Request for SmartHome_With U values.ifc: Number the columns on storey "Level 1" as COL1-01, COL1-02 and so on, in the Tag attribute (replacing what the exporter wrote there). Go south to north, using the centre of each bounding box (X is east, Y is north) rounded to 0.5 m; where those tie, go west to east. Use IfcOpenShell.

First a look at what the model holds.

```python
import ifcopenshell
import ifcopenshell.util.element
import ifcopenshell.util.placement

model = ifcopenshell.open("SmartHome_With U values.ifc")
print(model.schema)
storey = next(s for s in model.by_type("IfcBuildingStorey") if s.Name == "Level 1")
columns = [e for e in ifcopenshell.util.element.get_decomposition(storey) if e.is_a("IfcColumn")]
for e in sorted(columns, key=lambda e: e.id()):
    origin = ifcopenshell.util.placement.get_local_placement(e.ObjectPlacement)[:3, 3]
    print(e.id(), e.Tag, e.Name, origin.round(2) + 0.0, sep=" | ")
```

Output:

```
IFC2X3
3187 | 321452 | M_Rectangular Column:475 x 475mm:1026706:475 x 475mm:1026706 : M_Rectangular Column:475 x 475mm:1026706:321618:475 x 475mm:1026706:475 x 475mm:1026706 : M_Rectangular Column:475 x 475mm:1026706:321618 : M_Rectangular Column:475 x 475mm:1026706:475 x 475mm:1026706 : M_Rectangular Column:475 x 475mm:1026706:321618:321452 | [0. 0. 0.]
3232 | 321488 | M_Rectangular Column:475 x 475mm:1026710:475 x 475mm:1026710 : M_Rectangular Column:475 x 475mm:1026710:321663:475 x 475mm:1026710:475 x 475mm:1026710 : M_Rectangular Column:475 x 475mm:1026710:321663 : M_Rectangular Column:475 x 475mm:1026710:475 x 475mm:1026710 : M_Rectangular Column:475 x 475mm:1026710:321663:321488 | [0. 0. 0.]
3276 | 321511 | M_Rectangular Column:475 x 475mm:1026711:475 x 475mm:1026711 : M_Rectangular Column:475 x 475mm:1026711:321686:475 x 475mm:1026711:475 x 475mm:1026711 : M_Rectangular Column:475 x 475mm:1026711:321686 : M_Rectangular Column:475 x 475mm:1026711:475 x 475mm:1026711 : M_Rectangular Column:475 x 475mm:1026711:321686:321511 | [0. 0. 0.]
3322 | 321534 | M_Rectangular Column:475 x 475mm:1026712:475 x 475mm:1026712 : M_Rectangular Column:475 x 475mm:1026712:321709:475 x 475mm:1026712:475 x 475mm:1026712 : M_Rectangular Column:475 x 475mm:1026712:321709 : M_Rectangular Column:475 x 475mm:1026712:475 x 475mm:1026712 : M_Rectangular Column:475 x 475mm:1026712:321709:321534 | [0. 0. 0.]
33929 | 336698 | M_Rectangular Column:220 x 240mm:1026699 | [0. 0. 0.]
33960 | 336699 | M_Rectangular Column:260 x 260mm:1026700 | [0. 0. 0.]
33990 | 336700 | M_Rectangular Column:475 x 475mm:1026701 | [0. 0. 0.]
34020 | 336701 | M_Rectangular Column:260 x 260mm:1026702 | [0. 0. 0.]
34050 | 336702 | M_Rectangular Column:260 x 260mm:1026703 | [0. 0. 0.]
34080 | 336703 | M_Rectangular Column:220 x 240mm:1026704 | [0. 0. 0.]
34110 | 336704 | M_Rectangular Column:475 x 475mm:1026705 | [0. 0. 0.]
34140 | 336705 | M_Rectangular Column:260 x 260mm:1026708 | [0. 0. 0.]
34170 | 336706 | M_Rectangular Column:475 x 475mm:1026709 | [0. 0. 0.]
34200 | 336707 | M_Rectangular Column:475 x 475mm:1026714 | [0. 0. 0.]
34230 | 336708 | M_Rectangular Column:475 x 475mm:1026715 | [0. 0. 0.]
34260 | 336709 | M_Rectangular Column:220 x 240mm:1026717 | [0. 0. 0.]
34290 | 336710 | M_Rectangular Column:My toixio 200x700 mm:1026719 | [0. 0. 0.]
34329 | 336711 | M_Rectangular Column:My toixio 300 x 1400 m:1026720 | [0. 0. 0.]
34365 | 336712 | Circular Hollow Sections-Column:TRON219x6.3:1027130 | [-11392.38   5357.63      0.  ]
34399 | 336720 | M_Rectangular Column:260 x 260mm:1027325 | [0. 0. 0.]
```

```python
import ifcopenshell
import ifcopenshell.geom
import ifcopenshell.util.element
import ifcopenshell.util.shape

model = ifcopenshell.open("SmartHome_With U values.ifc")
settings = ifcopenshell.geom.settings()
settings.set("use-world-coords", True)


def centre(element):
    shape = ifcopenshell.geom.create_shape(settings, element)
    return ifcopenshell.util.shape.get_bbox_centroid(shape.geometry)


storey = next(s for s in model.by_type("IfcBuildingStorey") if s.Name == "Level 1")
columns = [e for e in ifcopenshell.util.element.get_decomposition(storey) if e.is_a("IfcColumn")]

# Insertion points can sit at a corner or the storey origin, so sort by the geometry (in metres).
centres = {e: centre(e) for e in columns}
columns.sort(key=lambda e: (round(centres[e][1] / 0.5), centres[e][0]))

for i, e in enumerate(columns, start=1):
    number = f"COL1-{i:02d}"
    e.Tag = number
    print(e.id(), number)

model.write("SmartHome_With U values_rev.ifc")
```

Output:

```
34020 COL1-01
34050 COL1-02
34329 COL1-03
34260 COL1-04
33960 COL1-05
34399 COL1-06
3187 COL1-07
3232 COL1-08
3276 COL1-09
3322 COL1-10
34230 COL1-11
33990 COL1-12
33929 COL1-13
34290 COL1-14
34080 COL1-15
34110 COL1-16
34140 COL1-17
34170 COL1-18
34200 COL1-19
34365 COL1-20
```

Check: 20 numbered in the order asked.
